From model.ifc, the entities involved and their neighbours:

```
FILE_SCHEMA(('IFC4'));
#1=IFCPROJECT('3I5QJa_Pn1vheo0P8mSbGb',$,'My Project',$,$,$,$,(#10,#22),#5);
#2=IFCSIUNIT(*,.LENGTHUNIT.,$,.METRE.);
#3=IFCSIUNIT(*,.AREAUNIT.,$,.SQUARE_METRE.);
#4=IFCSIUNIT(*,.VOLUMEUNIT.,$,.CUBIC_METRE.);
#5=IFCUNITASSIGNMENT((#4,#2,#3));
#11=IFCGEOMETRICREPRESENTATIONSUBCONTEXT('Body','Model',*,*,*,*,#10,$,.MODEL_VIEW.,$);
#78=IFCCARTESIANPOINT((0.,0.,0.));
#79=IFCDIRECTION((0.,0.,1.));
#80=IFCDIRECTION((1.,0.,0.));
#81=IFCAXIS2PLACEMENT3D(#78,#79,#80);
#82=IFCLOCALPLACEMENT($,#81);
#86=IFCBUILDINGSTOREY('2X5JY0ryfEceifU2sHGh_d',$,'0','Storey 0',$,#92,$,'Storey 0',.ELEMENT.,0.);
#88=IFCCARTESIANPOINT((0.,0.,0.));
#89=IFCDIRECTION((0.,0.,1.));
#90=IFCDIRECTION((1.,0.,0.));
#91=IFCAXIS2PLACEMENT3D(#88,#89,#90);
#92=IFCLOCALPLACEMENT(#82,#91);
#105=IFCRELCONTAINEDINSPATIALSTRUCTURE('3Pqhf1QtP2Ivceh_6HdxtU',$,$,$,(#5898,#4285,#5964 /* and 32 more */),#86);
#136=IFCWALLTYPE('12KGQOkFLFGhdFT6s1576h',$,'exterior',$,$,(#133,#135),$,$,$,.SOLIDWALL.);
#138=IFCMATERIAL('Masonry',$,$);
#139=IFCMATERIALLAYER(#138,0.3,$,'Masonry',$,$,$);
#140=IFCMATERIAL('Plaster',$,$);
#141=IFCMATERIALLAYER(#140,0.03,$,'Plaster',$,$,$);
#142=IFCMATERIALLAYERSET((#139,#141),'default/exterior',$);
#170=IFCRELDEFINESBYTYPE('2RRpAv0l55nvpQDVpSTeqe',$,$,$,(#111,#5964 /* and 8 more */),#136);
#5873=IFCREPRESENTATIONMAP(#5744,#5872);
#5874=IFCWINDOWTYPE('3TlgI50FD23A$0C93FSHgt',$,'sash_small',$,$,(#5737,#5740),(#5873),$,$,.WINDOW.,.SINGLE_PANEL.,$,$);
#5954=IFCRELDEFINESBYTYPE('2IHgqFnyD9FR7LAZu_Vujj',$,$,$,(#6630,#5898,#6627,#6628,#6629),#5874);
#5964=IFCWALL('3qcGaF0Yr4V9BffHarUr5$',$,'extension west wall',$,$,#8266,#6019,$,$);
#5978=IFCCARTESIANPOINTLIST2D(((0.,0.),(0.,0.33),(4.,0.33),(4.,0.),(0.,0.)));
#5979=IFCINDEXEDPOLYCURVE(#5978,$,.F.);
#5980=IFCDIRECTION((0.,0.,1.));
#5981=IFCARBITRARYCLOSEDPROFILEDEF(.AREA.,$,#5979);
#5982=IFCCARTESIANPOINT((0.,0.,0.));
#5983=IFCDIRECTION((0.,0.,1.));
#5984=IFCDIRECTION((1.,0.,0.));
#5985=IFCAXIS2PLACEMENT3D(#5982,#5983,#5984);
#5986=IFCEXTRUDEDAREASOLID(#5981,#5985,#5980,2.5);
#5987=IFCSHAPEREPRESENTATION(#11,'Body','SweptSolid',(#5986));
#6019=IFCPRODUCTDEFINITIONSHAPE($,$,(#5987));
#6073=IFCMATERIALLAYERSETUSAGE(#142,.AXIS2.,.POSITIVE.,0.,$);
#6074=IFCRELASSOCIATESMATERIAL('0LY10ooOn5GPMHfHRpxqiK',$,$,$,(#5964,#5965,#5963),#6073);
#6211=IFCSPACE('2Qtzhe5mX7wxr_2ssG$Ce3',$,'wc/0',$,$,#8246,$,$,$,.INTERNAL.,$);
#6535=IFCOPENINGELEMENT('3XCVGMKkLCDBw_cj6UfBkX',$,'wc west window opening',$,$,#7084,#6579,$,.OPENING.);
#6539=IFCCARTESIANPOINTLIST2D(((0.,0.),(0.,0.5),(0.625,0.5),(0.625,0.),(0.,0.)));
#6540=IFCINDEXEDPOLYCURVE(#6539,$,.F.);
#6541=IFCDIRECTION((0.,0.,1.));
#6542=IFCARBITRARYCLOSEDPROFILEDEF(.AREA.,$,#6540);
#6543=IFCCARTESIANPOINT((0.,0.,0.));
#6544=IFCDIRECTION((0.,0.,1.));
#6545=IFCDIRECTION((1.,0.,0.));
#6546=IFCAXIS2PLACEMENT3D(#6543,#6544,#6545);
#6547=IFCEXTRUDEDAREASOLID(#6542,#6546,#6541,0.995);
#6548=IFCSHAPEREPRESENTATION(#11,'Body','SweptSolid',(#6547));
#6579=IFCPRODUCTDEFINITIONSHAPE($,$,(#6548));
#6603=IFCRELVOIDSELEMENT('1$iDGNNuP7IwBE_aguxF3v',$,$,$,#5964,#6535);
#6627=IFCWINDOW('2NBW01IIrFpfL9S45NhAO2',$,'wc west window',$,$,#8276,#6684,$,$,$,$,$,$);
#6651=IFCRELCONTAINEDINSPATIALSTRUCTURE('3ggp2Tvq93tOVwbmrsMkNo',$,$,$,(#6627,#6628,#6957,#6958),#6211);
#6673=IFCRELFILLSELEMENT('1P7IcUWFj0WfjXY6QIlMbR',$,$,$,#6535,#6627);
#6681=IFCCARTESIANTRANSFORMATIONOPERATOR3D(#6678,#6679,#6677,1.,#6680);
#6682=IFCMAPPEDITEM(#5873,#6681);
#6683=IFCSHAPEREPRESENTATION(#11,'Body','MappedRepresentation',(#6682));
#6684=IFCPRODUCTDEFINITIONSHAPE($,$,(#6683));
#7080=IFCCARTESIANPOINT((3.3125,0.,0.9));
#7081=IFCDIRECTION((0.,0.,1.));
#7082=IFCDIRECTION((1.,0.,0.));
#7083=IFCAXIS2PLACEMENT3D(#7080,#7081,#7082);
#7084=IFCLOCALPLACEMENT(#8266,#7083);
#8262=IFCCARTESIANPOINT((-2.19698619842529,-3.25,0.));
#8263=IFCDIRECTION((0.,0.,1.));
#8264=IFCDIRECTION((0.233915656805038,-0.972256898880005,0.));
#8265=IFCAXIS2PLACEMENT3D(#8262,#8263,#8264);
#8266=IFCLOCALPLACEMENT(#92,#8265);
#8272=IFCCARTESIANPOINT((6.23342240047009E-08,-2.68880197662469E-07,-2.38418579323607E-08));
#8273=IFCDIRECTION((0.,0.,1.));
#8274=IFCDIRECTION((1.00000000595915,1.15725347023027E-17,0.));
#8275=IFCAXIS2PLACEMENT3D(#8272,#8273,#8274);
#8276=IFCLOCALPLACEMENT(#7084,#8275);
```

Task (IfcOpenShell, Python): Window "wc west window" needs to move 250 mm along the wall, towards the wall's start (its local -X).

```python
import ifcopenshell
import ifcopenshell.api.geometry
import ifcopenshell.util.placement
import ifcopenshell.util.unit

model = ifcopenshell.open("model.ifc")
unit_scale = ifcopenshell.util.unit.calculate_unit_scale(model)

window = model.by_guid("2NBW01IIrFpfL9S45NhAO2")
opening = window.FillsVoids[0].RelatingOpeningElement
wall = opening.VoidsElements[0].RelatingBuildingElement

wall_matrix = ifcopenshell.util.placement.get_local_placement(wall.ObjectPlacement)
shift = wall_matrix[:3, 0] * -0.25 / unit_scale
before = ifcopenshell.util.placement.get_local_placement(window.ObjectPlacement)[:3, 3].copy()

# The window is placed relative to its opening, so it follows when the opening moves.
matrix = ifcopenshell.util.placement.get_local_placement(opening.ObjectPlacement)
matrix[:3, 3] += shift
ifcopenshell.api.geometry.edit_object_placement(
    model, product=opening, matrix=matrix, is_si=False, should_transform_children=True
)

after = ifcopenshell.util.placement.get_local_placement(window.ObjectPlacement)[:3, 3]
print("window moved by", (after - before).round(3) + 0.0)

model.write("model_v2.ifc")
```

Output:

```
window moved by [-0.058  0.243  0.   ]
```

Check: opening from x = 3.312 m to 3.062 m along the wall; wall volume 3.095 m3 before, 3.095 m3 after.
